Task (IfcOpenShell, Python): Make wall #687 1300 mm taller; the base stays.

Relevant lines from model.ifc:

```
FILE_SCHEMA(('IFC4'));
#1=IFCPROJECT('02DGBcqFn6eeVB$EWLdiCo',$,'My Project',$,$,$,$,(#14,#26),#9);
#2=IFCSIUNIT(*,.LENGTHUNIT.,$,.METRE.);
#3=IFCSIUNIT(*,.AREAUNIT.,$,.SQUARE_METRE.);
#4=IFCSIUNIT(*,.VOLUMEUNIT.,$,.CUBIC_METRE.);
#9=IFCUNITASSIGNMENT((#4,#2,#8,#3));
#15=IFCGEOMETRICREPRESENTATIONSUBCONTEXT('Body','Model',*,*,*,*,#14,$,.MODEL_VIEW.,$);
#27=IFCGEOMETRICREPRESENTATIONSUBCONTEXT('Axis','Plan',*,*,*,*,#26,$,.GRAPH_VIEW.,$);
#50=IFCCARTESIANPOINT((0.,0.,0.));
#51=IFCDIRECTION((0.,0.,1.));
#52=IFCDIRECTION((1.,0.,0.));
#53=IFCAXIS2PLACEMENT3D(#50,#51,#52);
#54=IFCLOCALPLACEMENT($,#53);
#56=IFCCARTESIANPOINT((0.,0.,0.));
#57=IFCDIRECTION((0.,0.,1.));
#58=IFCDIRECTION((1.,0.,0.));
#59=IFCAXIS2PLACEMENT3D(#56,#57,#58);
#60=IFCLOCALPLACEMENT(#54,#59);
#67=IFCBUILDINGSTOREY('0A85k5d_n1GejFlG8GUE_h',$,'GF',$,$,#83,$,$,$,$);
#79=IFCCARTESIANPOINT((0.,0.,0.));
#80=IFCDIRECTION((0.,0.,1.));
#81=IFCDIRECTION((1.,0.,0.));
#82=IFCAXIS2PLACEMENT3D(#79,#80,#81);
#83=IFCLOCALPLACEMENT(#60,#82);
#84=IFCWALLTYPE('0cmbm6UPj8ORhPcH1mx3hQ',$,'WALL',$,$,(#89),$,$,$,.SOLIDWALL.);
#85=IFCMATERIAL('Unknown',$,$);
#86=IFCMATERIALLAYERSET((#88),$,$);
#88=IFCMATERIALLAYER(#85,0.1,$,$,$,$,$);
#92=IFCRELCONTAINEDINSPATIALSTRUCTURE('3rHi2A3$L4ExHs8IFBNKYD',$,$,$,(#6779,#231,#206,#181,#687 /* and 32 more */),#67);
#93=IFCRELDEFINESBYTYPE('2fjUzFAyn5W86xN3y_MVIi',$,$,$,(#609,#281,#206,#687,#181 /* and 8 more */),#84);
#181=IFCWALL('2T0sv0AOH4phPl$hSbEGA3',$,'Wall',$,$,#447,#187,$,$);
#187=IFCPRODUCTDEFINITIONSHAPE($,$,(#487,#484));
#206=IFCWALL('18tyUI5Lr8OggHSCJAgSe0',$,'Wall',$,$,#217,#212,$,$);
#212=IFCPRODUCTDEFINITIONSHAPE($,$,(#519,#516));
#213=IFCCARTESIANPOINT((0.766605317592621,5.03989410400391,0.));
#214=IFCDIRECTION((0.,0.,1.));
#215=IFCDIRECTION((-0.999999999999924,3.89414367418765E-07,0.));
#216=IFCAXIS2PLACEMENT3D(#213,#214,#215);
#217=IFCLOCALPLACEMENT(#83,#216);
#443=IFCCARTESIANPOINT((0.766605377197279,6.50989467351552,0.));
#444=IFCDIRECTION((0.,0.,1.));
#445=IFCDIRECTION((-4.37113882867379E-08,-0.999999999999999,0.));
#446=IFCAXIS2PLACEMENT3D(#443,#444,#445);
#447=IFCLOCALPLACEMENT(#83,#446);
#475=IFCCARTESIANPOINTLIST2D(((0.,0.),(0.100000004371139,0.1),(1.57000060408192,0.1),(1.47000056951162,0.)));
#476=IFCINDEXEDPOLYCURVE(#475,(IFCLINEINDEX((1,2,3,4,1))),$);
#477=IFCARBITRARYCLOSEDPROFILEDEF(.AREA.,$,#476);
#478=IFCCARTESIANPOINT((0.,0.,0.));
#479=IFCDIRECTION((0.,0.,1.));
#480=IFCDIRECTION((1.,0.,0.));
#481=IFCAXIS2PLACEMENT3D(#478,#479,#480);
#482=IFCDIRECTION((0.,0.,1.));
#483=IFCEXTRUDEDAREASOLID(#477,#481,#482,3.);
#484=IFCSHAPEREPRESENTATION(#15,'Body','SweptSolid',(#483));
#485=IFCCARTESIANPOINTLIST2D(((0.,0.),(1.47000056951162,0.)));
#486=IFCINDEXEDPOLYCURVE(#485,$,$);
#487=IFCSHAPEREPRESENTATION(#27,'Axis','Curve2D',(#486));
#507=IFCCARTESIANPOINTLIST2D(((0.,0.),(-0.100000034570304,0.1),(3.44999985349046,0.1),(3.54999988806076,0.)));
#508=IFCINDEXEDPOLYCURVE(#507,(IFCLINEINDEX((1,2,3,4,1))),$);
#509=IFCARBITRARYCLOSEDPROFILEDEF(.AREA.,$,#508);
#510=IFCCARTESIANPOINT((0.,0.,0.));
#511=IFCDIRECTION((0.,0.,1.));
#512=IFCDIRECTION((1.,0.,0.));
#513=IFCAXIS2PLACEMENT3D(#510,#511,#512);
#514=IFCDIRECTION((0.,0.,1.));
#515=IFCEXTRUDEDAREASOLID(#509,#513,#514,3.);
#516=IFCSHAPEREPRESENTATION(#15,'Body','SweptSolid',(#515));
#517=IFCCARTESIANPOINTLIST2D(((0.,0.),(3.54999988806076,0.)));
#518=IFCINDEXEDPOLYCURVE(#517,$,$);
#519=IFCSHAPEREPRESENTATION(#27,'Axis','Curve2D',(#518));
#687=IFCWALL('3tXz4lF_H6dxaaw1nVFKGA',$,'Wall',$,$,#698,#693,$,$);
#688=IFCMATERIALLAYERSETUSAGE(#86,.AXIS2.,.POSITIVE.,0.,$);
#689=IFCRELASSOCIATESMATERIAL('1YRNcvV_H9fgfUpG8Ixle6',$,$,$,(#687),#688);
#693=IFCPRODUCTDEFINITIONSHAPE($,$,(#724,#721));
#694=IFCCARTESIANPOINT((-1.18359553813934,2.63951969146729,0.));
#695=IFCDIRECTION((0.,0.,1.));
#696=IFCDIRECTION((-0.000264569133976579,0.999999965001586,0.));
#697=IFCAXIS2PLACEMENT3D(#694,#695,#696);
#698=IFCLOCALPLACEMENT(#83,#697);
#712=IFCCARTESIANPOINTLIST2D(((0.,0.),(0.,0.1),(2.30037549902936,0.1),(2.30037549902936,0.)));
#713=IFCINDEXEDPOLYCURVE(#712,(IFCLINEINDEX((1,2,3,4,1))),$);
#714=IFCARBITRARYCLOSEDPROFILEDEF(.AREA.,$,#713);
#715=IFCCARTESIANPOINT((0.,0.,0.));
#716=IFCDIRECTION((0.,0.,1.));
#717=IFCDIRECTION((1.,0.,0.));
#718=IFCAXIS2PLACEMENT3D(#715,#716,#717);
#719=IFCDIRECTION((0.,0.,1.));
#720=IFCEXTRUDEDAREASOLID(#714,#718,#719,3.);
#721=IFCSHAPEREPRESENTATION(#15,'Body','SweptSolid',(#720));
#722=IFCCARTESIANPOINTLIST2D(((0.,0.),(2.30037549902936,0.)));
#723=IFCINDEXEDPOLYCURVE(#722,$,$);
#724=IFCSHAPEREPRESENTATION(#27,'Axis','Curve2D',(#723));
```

```python
import ifcopenshell
import ifcopenshell.geom
import ifcopenshell.util.representation
import ifcopenshell.util.shape

model = ifcopenshell.open("model.ifc")
settings = ifcopenshell.geom.settings()


def volume(element):
    """Net volume in cubic metres, openings subtracted."""
    shape = ifcopenshell.geom.create_shape(settings, element)
    return ifcopenshell.util.shape.get_volume(shape.geometry)


wall = model.by_guid("3tXz4lF_H6dxaaw1nVFKGA")
before = volume(wall)

body = ifcopenshell.util.representation.get_representation(wall, "Model", "Body")
solid = body.Items[0]
old_height = solid.Depth
solid.Depth += 1.3
after = volume(wall)

print(f"height {old_height:g} -> {solid.Depth:g}, volume {before:.3f} -> {after:.3f} m3")

model.write("model_v2.ifc")
```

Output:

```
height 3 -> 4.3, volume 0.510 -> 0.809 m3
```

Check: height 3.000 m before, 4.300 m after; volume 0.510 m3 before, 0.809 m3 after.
